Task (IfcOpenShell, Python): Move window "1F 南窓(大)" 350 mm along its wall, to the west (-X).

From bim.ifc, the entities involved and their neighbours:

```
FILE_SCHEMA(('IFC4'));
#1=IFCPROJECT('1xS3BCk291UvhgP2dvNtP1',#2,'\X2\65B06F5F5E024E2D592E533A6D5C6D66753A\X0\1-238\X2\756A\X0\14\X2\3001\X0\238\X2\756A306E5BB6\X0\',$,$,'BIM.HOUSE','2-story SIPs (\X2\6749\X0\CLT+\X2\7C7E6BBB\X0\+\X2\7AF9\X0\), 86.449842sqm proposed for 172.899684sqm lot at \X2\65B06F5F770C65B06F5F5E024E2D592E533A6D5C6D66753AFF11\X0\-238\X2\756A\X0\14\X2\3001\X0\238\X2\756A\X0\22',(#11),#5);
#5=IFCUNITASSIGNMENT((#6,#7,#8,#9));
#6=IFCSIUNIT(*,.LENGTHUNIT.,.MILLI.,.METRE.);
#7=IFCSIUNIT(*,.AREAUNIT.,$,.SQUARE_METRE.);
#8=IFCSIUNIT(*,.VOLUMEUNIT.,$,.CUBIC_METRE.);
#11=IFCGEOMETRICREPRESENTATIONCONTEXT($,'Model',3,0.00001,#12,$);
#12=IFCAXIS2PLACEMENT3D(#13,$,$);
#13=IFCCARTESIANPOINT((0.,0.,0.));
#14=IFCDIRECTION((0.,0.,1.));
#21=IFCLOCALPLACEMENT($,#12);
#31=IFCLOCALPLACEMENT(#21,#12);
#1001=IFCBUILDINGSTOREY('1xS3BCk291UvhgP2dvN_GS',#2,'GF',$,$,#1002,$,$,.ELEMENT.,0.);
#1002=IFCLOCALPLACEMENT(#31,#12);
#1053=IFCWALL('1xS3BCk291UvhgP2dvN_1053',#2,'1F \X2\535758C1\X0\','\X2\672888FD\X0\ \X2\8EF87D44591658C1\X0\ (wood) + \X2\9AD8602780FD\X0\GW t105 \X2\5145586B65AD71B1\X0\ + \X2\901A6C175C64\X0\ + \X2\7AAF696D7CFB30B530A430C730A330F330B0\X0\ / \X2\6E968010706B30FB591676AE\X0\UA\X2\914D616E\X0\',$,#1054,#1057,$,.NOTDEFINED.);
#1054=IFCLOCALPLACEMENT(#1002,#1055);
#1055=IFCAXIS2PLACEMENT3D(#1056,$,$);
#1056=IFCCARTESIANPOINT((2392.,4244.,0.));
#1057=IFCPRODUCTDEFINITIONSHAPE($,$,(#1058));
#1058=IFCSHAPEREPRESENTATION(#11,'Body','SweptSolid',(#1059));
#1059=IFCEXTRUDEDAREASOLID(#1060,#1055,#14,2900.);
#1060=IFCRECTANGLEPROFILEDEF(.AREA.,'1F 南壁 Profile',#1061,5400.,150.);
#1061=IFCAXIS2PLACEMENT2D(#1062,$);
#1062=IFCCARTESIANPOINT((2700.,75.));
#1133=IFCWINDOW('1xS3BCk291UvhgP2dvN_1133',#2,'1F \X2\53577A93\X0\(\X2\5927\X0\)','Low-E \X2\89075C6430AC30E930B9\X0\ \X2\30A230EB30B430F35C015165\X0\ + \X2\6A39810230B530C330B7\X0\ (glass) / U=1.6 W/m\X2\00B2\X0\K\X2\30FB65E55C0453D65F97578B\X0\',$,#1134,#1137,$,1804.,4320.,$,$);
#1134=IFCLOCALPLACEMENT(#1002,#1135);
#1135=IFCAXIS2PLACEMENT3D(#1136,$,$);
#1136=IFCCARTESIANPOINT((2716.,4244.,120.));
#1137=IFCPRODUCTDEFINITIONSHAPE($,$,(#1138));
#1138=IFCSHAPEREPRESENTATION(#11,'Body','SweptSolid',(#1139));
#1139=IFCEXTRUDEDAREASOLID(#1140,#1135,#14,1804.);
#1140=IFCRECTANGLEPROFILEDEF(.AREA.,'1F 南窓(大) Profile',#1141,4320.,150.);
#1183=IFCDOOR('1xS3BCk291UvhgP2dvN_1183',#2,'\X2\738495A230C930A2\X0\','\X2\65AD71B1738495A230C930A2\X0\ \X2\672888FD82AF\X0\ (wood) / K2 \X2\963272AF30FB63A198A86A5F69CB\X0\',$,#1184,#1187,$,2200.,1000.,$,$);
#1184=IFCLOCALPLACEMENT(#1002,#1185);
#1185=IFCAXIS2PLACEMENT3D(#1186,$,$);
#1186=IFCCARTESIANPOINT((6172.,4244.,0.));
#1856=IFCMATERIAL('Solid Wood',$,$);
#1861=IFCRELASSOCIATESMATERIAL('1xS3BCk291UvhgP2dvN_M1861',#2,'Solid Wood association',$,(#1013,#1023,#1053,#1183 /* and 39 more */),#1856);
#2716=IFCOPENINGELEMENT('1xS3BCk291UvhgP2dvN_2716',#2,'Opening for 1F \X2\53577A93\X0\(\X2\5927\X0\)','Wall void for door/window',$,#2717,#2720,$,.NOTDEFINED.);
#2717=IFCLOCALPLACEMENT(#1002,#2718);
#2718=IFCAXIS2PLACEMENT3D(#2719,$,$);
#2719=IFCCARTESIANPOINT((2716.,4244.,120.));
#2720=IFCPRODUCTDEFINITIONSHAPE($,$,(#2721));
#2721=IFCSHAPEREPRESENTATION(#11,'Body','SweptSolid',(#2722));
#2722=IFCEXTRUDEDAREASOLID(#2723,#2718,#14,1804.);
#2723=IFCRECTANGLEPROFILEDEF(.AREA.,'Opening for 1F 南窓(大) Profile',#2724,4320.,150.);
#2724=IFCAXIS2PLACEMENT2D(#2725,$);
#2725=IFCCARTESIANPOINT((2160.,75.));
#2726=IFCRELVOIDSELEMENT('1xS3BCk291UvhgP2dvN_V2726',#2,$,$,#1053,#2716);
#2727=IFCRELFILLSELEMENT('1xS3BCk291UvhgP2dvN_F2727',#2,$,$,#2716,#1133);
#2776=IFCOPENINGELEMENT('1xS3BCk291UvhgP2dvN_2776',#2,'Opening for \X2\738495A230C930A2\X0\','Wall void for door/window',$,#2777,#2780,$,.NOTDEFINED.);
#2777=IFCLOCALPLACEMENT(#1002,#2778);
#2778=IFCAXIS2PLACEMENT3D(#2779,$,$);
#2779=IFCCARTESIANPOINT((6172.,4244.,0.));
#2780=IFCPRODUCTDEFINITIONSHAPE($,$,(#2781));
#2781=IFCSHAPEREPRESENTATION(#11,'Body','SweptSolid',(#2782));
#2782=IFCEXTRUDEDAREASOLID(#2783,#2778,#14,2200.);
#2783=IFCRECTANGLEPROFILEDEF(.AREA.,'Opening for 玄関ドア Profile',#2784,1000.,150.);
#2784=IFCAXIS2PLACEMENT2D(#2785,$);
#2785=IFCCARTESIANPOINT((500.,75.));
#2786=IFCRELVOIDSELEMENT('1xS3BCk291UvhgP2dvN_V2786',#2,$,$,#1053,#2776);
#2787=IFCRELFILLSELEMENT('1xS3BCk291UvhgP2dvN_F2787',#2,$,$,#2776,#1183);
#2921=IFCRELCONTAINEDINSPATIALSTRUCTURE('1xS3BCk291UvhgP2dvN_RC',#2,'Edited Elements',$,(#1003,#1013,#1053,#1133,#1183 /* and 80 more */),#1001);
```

```python
import ifcopenshell
import ifcopenshell.api.geometry
import ifcopenshell.util.placement

model = ifcopenshell.open("bim.ifc")

window = model.by_guid("1xS3BCk291UvhgP2dvN_1133")
opening = window.FillsVoids[0].RelatingOpeningElement
wall = opening.VoidsElements[0].RelatingBuildingElement

wall_matrix = ifcopenshell.util.placement.get_local_placement(wall.ObjectPlacement)
shift = wall_matrix[:3, 0] * -350.0
before = ifcopenshell.util.placement.get_local_placement(window.ObjectPlacement)[:3, 3].copy()

# The window is not placed relative to its opening, so move both.
for product in (opening, window):
    matrix = ifcopenshell.util.placement.get_local_placement(product.ObjectPlacement)
    matrix[:3, 3] += shift
    ifcopenshell.api.geometry.edit_object_placement(model, product=product, matrix=matrix, is_si=False)

after = ifcopenshell.util.placement.get_local_placement(window.ObjectPlacement)[:3, 3]
print("window moved by", (after - before).round(3) + 0.0)

model.write("bim_rev.ifc")
```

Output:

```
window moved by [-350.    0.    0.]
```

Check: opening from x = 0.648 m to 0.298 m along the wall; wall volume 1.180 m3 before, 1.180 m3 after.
